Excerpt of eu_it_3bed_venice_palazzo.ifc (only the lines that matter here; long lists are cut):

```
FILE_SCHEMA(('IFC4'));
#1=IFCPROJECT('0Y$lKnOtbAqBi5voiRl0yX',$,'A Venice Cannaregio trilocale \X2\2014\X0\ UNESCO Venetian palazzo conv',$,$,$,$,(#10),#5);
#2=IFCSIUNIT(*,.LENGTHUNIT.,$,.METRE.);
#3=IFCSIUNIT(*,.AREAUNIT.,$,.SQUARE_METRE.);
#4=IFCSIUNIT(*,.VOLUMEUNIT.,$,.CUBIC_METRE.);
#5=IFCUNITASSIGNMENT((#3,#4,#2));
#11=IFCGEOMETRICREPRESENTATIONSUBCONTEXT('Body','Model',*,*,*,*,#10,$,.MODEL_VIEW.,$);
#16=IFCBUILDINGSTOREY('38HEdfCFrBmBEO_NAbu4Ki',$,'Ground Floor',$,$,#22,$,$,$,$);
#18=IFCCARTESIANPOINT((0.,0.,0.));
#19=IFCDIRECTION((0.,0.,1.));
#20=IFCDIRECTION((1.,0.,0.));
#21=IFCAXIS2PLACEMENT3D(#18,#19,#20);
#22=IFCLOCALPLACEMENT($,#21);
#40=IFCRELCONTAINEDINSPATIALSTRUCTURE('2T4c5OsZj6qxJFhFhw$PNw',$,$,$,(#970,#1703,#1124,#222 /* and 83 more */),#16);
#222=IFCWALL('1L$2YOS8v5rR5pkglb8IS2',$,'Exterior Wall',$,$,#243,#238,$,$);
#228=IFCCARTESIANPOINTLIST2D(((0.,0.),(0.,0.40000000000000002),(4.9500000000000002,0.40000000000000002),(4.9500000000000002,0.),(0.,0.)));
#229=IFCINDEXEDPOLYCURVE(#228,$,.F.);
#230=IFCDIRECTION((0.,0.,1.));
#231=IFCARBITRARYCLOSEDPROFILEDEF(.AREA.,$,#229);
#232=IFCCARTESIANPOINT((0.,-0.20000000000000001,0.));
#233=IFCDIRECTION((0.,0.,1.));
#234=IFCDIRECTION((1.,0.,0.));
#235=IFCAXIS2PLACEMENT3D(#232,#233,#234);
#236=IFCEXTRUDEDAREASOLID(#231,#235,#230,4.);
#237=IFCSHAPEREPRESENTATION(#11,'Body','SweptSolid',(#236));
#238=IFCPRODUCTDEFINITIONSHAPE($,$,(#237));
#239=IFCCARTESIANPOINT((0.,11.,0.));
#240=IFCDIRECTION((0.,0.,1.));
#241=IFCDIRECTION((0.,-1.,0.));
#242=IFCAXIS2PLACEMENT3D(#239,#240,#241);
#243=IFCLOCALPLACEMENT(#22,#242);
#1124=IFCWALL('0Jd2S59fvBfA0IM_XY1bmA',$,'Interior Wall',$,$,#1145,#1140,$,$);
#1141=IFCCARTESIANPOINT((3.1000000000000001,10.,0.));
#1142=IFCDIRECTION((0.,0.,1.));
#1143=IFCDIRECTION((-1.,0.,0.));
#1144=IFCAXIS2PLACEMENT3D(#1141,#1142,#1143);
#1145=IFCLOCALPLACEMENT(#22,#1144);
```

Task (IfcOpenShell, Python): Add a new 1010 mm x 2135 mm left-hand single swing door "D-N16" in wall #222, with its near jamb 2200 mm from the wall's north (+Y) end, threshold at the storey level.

```python
import numpy as np
import ifcopenshell
import ifcopenshell.api.feature
import ifcopenshell.api.geometry
import ifcopenshell.api.root
import ifcopenshell.api.spatial
import ifcopenshell.geom
import ifcopenshell.util.element
import ifcopenshell.util.placement
import ifcopenshell.util.representation
import ifcopenshell.util.shape
import ifcopenshell.util.unit

model = ifcopenshell.open("eu_it_3bed_venice_palazzo.ifc")
unit_scale = ifcopenshell.util.unit.calculate_unit_scale(model)
settings = ifcopenshell.geom.settings()


def volume(element):
    """Net volume in cubic metres, openings subtracted."""
    shape = ifcopenshell.geom.create_shape(settings, element)
    return ifcopenshell.util.shape.get_volume(shape.geometry)


wall = model.by_guid("1L$2YOS8v5rR5pkglb8IS2")
storey = ifcopenshell.util.element.get_container(wall, ifc_class="IfcBuildingStorey")
context = ifcopenshell.util.representation.get_context(model, "Model", "Body", "MODEL_VIEW")
before = volume(wall)

width, height, from_end, sill = 1.01, 2.135, 2.2, 0.0  # metres

# The wall runs along its own X axis, and the end named is its -X end.
wall_shape = ifcopenshell.geom.create_shape(settings, wall)
x, y, z = ifcopenshell.util.shape.get_vertices(wall_shape.geometry).T
start = x.min() + from_end
face, thickness = float(y.min()), float(y.max() - y.min())
wall_matrix = ifcopenshell.util.placement.get_local_placement(wall.ObjectPlacement)
level = ifcopenshell.util.placement.get_local_placement(storey.ObjectPlacement)[2, 3]


def in_wall(x, y):
    """Placement at x, y metres in the wall's axes, at sill height."""
    matrix = wall_matrix.copy()
    matrix[:, 3] = wall_matrix @ np.array([x / unit_scale, y / unit_scale, 0.0, 1.0])
    matrix[2, 3] = level + sill / unit_scale
    return matrix


# Opening: a box that overshoots both wall faces by 50 mm.
opening = ifcopenshell.api.root.create_entity(model, ifc_class="IfcOpeningElement", predefined_type="OPENING")
box = ifcopenshell.api.geometry.add_wall_representation(
    model, context=context, length=width, height=height, thickness=thickness + 0.1
)
ifcopenshell.api.geometry.assign_representation(model, product=opening, representation=box)
ifcopenshell.api.geometry.edit_object_placement(model, product=opening, matrix=in_wall(start, face - 0.05), is_si=False)
ifcopenshell.api.feature.add_feature(model, feature=opening, element=wall)

door = ifcopenshell.api.root.create_entity(model, ifc_class="IfcDoor", name="D-N16", predefined_type="DOOR")
door.OverallWidth, door.OverallHeight = width / unit_scale, height / unit_scale
door.OperationType = "SINGLE_SWING_LEFT"
body = ifcopenshell.api.geometry.add_door_representation(
    model,
    context=context,
    overall_width=door.OverallWidth,
    overall_height=door.OverallHeight,
    operation_type="SINGLE_SWING_LEFT",
    lining_properties={"LiningDepth": thickness / unit_scale, "ThresholdDepth": thickness / unit_scale},
)
ifcopenshell.api.geometry.assign_representation(model, product=door, representation=body)
ifcopenshell.api.spatial.assign_container(model, products=[door], relating_structure=storey)
ifcopenshell.api.feature.add_filling(model, opening=opening, element=door)

# The lining spans the wall, so the door starts at the wall face.
ifcopenshell.api.geometry.edit_object_placement(model, product=door, matrix=in_wall(start, face), is_si=False)

after = volume(wall)

print(f"wall volume {before:.3f} -> {after:.3f} m3")

model.write("eu_it_3bed_venice_palazzo_v2.ifc")
```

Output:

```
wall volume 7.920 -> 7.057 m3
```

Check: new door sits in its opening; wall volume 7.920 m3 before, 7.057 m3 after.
